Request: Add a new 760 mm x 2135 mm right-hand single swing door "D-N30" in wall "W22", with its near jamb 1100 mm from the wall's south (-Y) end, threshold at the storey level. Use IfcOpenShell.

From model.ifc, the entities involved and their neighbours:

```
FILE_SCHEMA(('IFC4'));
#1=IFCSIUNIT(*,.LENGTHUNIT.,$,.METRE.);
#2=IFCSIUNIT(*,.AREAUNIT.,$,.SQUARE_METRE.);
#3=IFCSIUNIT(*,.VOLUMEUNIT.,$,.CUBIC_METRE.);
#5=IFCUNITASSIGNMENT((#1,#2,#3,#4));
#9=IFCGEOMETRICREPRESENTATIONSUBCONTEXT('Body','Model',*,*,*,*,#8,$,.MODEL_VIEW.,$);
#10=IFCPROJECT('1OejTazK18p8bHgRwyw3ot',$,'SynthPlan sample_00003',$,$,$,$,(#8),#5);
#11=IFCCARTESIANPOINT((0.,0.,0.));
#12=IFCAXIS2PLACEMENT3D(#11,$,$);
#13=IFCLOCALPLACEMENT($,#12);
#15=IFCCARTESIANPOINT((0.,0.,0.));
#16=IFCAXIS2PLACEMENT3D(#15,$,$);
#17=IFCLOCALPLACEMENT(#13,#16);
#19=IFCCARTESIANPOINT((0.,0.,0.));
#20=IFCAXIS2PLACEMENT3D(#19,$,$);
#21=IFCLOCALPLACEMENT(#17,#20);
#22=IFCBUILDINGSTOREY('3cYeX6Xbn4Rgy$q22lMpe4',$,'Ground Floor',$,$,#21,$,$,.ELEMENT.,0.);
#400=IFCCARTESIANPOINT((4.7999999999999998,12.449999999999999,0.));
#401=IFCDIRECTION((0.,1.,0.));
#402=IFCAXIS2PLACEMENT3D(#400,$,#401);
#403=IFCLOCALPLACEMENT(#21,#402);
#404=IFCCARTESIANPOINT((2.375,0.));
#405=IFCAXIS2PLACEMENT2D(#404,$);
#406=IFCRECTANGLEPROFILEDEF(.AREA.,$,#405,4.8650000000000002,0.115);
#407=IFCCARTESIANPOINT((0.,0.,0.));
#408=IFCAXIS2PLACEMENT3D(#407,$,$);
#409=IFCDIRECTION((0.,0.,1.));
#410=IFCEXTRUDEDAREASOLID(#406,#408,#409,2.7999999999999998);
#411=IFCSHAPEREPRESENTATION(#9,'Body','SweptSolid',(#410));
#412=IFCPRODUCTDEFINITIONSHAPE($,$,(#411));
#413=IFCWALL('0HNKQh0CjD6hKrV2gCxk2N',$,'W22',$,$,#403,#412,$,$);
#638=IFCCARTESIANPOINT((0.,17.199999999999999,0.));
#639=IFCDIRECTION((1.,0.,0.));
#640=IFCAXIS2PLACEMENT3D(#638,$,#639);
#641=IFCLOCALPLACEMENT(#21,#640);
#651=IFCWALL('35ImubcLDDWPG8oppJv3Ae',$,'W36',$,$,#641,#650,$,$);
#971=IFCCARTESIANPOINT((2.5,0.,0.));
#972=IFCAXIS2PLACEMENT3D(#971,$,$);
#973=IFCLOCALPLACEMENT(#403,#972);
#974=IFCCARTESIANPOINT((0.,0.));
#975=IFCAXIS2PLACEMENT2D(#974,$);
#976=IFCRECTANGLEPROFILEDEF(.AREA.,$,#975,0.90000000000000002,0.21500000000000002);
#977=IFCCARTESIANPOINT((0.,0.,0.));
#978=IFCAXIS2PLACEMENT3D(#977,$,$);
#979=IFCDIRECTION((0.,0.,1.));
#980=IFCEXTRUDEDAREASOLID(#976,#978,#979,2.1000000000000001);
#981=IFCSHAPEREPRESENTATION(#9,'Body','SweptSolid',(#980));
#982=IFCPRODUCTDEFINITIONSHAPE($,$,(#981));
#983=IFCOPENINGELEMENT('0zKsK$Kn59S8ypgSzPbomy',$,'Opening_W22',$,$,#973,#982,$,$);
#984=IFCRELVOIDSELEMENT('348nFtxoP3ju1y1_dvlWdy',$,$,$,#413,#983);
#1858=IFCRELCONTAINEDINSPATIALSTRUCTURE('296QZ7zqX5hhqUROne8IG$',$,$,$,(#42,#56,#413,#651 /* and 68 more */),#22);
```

```python
import numpy as np
import ifcopenshell
import ifcopenshell.api.feature
import ifcopenshell.api.geometry
import ifcopenshell.api.root
import ifcopenshell.api.spatial
import ifcopenshell.geom
import ifcopenshell.util.element
import ifcopenshell.util.placement
import ifcopenshell.util.representation
import ifcopenshell.util.shape
import ifcopenshell.util.unit

model = ifcopenshell.open("model.ifc")
unit_scale = ifcopenshell.util.unit.calculate_unit_scale(model)
settings = ifcopenshell.geom.settings()


def volume(element):
    """Net volume in cubic metres, openings subtracted."""
    shape = ifcopenshell.geom.create_shape(settings, element)
    return ifcopenshell.util.shape.get_volume(shape.geometry)


wall = model.by_id(413)
storey = ifcopenshell.util.element.get_container(wall, ifc_class="IfcBuildingStorey")
context = ifcopenshell.util.representation.get_context(model, "Model", "Body", "MODEL_VIEW")
before = volume(wall)

width, height, from_end, sill = 0.76, 2.135, 1.1, 0.0  # metres

# The wall runs along its own X axis, and the end named is its -X end.
wall_shape = ifcopenshell.geom.create_shape(settings, wall)
x, y, z = ifcopenshell.util.shape.get_vertices(wall_shape.geometry).T
start = x.min() + from_end
face, thickness = float(y.min()), float(y.max() - y.min())
wall_matrix = ifcopenshell.util.placement.get_local_placement(wall.ObjectPlacement)
level = ifcopenshell.util.placement.get_local_placement(storey.ObjectPlacement)[2, 3]


def in_wall(x, y):
    """Placement at x, y metres in the wall's axes, at sill height."""
    matrix = wall_matrix.copy()
    matrix[:, 3] = wall_matrix @ np.array([x / unit_scale, y / unit_scale, 0.0, 1.0])
    matrix[2, 3] = level + sill / unit_scale
    return matrix


# Opening: a box that overshoots both wall faces by 50 mm.
opening = ifcopenshell.api.root.create_entity(model, ifc_class="IfcOpeningElement", predefined_type="OPENING")
box = ifcopenshell.api.geometry.add_wall_representation(
    model, context=context, length=width, height=height, thickness=thickness + 0.1
)
ifcopenshell.api.geometry.assign_representation(model, product=opening, representation=box)
ifcopenshell.api.geometry.edit_object_placement(model, product=opening, matrix=in_wall(start, face - 0.05), is_si=False)
ifcopenshell.api.feature.add_feature(model, feature=opening, element=wall)

door = ifcopenshell.api.root.create_entity(model, ifc_class="IfcDoor", name="D-N30", predefined_type="DOOR")
door.OverallWidth, door.OverallHeight = width / unit_scale, height / unit_scale
door.OperationType = "SINGLE_SWING_RIGHT"
body = ifcopenshell.api.geometry.add_door_representation(
    model,
    context=context,
    overall_width=door.OverallWidth,
    overall_height=door.OverallHeight,
    operation_type="SINGLE_SWING_RIGHT",
    lining_properties={"LiningDepth": thickness / unit_scale, "ThresholdDepth": thickness / unit_scale},
)
ifcopenshell.api.geometry.assign_representation(model, product=door, representation=body)
ifcopenshell.api.spatial.assign_container(model, products=[door], relating_structure=storey)
ifcopenshell.api.feature.add_filling(model, opening=opening, element=door)

# The lining spans the wall, so the door starts at the wall face.
ifcopenshell.api.geometry.edit_object_placement(model, product=door, matrix=in_wall(start, face), is_si=False)

after = volume(wall)

print(f"wall volume {before:.3f} -> {after:.3f} m3")

model.write("model-out.ifc")
```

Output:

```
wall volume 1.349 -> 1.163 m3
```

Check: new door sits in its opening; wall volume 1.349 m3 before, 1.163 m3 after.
